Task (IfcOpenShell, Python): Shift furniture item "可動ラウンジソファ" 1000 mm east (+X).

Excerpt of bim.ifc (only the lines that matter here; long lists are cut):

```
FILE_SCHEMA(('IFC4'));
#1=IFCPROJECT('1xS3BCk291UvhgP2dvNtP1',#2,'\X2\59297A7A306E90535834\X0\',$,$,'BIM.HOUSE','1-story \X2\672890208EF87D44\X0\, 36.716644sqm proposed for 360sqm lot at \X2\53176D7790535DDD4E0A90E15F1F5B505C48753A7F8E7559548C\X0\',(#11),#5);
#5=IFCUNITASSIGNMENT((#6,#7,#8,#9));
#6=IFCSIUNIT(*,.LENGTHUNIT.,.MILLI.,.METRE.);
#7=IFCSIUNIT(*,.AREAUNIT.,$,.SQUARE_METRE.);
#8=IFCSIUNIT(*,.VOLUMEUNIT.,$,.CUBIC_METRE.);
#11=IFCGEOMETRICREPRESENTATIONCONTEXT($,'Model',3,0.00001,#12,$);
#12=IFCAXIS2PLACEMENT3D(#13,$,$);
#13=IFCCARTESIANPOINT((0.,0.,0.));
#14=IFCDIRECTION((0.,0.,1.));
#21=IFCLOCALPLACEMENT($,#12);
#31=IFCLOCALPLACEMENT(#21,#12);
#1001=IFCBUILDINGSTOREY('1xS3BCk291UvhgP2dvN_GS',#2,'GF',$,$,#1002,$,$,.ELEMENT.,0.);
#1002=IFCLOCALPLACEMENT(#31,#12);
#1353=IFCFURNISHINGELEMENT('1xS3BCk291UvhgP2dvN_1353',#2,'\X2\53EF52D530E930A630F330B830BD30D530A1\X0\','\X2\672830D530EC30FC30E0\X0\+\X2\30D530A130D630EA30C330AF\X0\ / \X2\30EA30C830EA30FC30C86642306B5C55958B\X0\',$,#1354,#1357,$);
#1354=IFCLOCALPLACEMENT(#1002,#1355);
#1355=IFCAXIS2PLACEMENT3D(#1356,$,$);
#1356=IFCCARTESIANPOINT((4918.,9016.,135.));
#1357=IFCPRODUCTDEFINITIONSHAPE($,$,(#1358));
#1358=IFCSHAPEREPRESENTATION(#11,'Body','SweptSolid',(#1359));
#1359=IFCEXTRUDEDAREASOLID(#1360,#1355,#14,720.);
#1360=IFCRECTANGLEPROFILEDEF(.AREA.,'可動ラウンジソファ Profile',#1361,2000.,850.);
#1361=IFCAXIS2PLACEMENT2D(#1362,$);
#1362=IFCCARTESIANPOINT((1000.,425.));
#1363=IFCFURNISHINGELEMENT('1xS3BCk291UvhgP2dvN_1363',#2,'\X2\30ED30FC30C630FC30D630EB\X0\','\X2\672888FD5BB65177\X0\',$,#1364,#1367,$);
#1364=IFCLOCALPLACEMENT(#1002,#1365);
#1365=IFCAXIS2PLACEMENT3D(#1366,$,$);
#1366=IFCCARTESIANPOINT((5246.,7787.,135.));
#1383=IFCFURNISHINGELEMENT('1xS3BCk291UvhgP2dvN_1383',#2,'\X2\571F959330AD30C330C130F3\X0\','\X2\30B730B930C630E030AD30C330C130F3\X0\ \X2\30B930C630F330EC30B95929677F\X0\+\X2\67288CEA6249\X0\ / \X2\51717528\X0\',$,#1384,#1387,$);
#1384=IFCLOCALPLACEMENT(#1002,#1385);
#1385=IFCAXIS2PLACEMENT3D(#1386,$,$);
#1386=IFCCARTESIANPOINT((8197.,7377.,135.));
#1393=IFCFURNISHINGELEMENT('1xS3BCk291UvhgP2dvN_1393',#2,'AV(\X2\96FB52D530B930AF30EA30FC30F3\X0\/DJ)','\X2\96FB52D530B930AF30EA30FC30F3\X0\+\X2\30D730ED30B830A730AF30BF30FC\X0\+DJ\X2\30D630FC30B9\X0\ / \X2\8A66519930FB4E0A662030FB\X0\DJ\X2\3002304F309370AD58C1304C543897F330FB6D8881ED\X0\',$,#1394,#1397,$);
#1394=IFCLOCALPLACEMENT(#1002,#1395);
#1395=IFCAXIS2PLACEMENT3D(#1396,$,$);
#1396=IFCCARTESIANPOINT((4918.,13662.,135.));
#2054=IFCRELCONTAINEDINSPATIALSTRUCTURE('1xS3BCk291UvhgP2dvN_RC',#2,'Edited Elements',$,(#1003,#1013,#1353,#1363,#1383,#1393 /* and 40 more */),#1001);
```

```python
import ifcopenshell
import ifcopenshell.api.geometry
import ifcopenshell.util.placement

model = ifcopenshell.open("bim.ifc")

item = model.by_guid("1xS3BCk291UvhgP2dvN_1353")
matrix = ifcopenshell.util.placement.get_local_placement(item.ObjectPlacement)
matrix[0, 3] += 1000.0
ifcopenshell.api.geometry.edit_object_placement(model, product=item, matrix=matrix, is_si=False)

print(ifcopenshell.util.placement.get_local_placement(item.ObjectPlacement).round(3) + 0.0)

model.write("bim-out.ifc")
```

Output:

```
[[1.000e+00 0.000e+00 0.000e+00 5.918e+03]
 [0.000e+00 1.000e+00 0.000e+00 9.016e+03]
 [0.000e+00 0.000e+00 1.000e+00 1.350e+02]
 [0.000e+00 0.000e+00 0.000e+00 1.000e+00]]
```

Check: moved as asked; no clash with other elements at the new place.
